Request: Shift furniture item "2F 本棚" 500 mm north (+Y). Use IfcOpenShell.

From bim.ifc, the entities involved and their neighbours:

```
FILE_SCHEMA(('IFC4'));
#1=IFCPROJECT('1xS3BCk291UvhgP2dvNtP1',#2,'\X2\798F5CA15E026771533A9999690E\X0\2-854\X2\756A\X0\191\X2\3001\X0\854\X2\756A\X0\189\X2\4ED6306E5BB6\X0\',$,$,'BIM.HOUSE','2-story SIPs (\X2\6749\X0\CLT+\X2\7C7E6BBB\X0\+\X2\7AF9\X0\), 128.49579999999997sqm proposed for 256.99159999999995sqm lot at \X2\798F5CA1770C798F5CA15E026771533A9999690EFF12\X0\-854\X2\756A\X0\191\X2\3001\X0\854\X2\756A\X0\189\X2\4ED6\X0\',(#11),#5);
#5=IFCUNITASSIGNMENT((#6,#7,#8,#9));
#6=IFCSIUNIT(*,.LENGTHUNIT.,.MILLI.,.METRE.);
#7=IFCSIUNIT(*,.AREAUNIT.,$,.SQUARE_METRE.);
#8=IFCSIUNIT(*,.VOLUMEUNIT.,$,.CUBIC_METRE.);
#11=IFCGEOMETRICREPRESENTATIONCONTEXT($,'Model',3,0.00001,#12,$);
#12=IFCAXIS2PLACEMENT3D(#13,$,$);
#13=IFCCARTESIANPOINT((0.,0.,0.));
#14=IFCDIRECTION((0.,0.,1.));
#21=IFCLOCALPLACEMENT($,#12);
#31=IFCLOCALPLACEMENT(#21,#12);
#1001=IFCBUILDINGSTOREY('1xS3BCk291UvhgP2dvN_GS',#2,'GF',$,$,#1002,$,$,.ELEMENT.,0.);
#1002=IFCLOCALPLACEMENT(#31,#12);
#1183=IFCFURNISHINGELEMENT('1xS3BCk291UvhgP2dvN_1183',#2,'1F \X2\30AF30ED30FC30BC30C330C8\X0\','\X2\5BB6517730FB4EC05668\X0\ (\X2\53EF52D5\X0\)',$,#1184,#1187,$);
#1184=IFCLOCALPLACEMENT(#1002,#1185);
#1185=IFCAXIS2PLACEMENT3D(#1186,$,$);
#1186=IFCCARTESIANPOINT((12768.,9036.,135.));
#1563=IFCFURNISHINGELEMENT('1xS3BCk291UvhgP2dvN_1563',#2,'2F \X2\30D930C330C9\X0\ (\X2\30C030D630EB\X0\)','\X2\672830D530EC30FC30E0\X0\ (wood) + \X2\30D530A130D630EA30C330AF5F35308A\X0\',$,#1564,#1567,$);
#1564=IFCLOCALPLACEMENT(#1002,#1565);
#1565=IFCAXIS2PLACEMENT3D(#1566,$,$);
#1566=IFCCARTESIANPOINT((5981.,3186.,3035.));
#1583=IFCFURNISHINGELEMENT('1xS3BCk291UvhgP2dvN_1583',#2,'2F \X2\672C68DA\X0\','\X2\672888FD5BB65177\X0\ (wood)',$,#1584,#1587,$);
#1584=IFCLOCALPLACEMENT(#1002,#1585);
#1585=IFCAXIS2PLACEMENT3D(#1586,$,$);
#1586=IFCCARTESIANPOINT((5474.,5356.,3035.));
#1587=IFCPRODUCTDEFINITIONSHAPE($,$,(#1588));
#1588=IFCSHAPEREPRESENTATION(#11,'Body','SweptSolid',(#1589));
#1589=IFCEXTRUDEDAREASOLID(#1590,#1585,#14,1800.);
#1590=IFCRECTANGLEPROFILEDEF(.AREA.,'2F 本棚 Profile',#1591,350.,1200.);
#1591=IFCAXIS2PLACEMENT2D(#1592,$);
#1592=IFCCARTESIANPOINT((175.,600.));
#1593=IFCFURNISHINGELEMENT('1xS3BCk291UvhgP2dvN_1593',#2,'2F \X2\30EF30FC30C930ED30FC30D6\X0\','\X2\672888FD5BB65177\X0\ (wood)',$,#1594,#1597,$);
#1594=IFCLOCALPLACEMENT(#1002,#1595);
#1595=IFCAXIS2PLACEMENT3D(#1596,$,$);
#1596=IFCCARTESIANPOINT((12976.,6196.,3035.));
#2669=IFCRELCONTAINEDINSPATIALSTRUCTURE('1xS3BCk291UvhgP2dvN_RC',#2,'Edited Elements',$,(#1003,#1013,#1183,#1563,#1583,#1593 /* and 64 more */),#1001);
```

```python
import ifcopenshell
import ifcopenshell.api.geometry
import ifcopenshell.util.placement
import ifcopenshell.util.unit

model = ifcopenshell.open("bim.ifc")
unit_scale = ifcopenshell.util.unit.calculate_unit_scale(model)

item = model.by_id(1583)
matrix = ifcopenshell.util.placement.get_local_placement(item.ObjectPlacement)
matrix[1, 3] += 0.5 / unit_scale
ifcopenshell.api.geometry.edit_object_placement(model, product=item, matrix=matrix, is_si=False)

print(ifcopenshell.util.placement.get_local_placement(item.ObjectPlacement).round(3) + 0.0)

model.write("bim_edited.ifc")
```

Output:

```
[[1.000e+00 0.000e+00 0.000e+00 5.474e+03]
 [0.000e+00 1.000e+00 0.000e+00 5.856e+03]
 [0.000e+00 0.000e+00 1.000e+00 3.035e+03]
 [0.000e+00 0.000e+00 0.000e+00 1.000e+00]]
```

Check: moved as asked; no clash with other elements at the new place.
